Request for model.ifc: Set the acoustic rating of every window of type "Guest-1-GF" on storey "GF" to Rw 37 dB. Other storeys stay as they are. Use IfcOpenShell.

First a look at what the model holds.

```python
import ifcopenshell
import ifcopenshell.util.element

model = ifcopenshell.open("model.ifc")
print(model.schema)
storey = next(s for s in model.by_type("IfcBuildingStorey") if s.Name == "GF")
windows = [e for e in ifcopenshell.util.element.get_decomposition(storey) if e.is_a("IfcWindow")]
seen = {}
for e in windows:
    element_type = ifcopenshell.util.element.get_type(e)
    key = (element_type.Name if element_type != e and element_type else None, ifcopenshell.util.element.get_pset(e, "Pset_WindowCommon", "AcousticRating"))
    seen[key] = seen.get(key, 0) + 1
for (name, value), count in sorted(seen.items(), key=str):
    print(count, "x", name, "|", value)
```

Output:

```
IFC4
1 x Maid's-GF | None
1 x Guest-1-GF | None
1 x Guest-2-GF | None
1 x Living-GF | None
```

```python
import ifcopenshell
import ifcopenshell.api.pset
import ifcopenshell.util.element

model = ifcopenshell.open("model.ifc")

storey = next(s for s in model.by_type("IfcBuildingStorey") if s.Name == "GF")
windows = [e for e in ifcopenshell.util.element.get_decomposition(storey) if e.is_a("IfcWindow")]

count = 0
for e in windows:
    element_type = ifcopenshell.util.element.get_type(e)
    if element_type in (None, e) or element_type.Name != "Guest-1-GF":
        continue
    # add_pset returns the element's existing set when there is one.
    pset = ifcopenshell.api.pset.add_pset(model, product=e, name="Pset_WindowCommon")
    ifcopenshell.api.pset.edit_pset(model, pset=pset, properties={"AcousticRating": "Rw 37 dB"})
    count += 1

print(count, "windows updated")

model.write("model_rev.ifc")
```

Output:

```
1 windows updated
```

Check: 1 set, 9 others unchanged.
